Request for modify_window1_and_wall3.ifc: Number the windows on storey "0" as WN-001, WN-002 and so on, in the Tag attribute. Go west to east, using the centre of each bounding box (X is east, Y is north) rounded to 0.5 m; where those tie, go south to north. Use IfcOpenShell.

First a look at what the model holds.

```python
import ifcopenshell
import ifcopenshell.util.element
import ifcopenshell.util.placement

model = ifcopenshell.open("modify_window1_and_wall3.ifc")
print(model.schema)
storey = next(s for s in model.by_type("IfcBuildingStorey") if s.Name == "0")
windows = [e for e in ifcopenshell.util.element.get_decomposition(storey) if e.is_a("IfcWindow")]
for e in sorted(windows, key=lambda e: e.id()):
    origin = ifcopenshell.util.placement.get_local_placement(e.ObjectPlacement)[:3, 3]
    print(e.id(), e.Tag, e.Name, origin.round(2) + 0.0, sep=" | ")
```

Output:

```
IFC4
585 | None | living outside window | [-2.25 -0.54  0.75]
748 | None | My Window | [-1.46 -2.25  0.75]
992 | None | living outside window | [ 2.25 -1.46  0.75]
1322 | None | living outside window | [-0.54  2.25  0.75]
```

```python
import ifcopenshell
import ifcopenshell.geom
import ifcopenshell.util.element
import ifcopenshell.util.shape

model = ifcopenshell.open("modify_window1_and_wall3.ifc")
settings = ifcopenshell.geom.settings()
settings.set("use-world-coords", True)


def centre(element):
    shape = ifcopenshell.geom.create_shape(settings, element)
    return ifcopenshell.util.shape.get_bbox_centroid(shape.geometry)


storey = next(s for s in model.by_type("IfcBuildingStorey") if s.Name == "0")
windows = [e for e in ifcopenshell.util.element.get_decomposition(storey) if e.is_a("IfcWindow")]

# Insertion points can sit at a corner or the storey origin, so sort by the geometry (in metres).
centres = {e: centre(e) for e in windows}
windows.sort(key=lambda e: (round(centres[e][0] / 0.5), centres[e][1]))

for i, e in enumerate(windows, start=1):
    number = f"WN-0{i:02d}"
    e.Tag = number
    print(e.id(), number)

model.write("modify_window1_and_wall3_rev.ifc")
```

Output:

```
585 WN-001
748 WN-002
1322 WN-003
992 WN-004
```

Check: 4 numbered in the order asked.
